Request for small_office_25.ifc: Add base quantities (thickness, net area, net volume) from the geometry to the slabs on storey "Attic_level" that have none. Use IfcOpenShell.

First a look at what the model holds.

```python
import ifcopenshell
import ifcopenshell.util.element
import ifcopenshell.util.unit

model = ifcopenshell.open("small_office_25.ifc")
print(model.schema)
for unit_type in ("LENGTHUNIT", "AREAUNIT", "VOLUMEUNIT"):
    print(unit_type, ifcopenshell.util.unit.calculate_unit_scale(model, unit_type))
storey = next(s for s in model.by_type("IfcBuildingStorey") if s.Name == "Attic_level")
slabs = [e for e in ifcopenshell.util.element.get_decomposition(storey) if e.is_a("IfcSlab")]
for e in sorted(slabs, key=lambda e: e.id()):
    print(e.id(), e.is_a(), e.Name, list(ifcopenshell.util.element.get_psets(e, qtos_only=True)), sep=" | ")
```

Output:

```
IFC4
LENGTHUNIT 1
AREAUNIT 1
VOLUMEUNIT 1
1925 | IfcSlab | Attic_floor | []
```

```python
import ifcopenshell
import ifcopenshell.api.pset
import ifcopenshell.geom
import ifcopenshell.util.element
import ifcopenshell.util.shape
import ifcopenshell.util.unit

model = ifcopenshell.open("small_office_25.ifc")
unit_scale = ifcopenshell.util.unit.calculate_unit_scale(model)
area_scale = ifcopenshell.util.unit.calculate_unit_scale(model, "AREAUNIT")
volume_scale = ifcopenshell.util.unit.calculate_unit_scale(model, "VOLUMEUNIT")
settings = ifcopenshell.geom.settings()

storey = next(s for s in model.by_type("IfcBuildingStorey") if s.Name == "Attic_level")
slabs = [e for e in ifcopenshell.util.element.get_decomposition(storey) if e.is_a("IfcSlab")]

for e in sorted(slabs, key=lambda e: e.id()):
    if ifcopenshell.util.element.get_psets(e, qtos_only=True, should_inherit=False):
        continue
    # Geometry comes back in metres, in the element's own axes.
    shape = ifcopenshell.geom.create_shape(settings, e)
    values = {
        "Width": ifcopenshell.util.shape.get_z(shape.geometry) / unit_scale,
        "NetArea": ifcopenshell.util.shape.get_footprint_area(shape.geometry) / area_scale,
        "NetVolume": ifcopenshell.util.shape.get_volume(shape.geometry) / volume_scale,
    }
    qto = ifcopenshell.api.pset.add_qto(model, product=e, name="Qto_SlabBaseQuantities")
    ifcopenshell.api.pset.edit_qto(model, qto=qto, properties=values)
    print(e.id(), {k: round(v, 3) for k, v in values.items()})

model.write("small_office_25_updated.ifc")
```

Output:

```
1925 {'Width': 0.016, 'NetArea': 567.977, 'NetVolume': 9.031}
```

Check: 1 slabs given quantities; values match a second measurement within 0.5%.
